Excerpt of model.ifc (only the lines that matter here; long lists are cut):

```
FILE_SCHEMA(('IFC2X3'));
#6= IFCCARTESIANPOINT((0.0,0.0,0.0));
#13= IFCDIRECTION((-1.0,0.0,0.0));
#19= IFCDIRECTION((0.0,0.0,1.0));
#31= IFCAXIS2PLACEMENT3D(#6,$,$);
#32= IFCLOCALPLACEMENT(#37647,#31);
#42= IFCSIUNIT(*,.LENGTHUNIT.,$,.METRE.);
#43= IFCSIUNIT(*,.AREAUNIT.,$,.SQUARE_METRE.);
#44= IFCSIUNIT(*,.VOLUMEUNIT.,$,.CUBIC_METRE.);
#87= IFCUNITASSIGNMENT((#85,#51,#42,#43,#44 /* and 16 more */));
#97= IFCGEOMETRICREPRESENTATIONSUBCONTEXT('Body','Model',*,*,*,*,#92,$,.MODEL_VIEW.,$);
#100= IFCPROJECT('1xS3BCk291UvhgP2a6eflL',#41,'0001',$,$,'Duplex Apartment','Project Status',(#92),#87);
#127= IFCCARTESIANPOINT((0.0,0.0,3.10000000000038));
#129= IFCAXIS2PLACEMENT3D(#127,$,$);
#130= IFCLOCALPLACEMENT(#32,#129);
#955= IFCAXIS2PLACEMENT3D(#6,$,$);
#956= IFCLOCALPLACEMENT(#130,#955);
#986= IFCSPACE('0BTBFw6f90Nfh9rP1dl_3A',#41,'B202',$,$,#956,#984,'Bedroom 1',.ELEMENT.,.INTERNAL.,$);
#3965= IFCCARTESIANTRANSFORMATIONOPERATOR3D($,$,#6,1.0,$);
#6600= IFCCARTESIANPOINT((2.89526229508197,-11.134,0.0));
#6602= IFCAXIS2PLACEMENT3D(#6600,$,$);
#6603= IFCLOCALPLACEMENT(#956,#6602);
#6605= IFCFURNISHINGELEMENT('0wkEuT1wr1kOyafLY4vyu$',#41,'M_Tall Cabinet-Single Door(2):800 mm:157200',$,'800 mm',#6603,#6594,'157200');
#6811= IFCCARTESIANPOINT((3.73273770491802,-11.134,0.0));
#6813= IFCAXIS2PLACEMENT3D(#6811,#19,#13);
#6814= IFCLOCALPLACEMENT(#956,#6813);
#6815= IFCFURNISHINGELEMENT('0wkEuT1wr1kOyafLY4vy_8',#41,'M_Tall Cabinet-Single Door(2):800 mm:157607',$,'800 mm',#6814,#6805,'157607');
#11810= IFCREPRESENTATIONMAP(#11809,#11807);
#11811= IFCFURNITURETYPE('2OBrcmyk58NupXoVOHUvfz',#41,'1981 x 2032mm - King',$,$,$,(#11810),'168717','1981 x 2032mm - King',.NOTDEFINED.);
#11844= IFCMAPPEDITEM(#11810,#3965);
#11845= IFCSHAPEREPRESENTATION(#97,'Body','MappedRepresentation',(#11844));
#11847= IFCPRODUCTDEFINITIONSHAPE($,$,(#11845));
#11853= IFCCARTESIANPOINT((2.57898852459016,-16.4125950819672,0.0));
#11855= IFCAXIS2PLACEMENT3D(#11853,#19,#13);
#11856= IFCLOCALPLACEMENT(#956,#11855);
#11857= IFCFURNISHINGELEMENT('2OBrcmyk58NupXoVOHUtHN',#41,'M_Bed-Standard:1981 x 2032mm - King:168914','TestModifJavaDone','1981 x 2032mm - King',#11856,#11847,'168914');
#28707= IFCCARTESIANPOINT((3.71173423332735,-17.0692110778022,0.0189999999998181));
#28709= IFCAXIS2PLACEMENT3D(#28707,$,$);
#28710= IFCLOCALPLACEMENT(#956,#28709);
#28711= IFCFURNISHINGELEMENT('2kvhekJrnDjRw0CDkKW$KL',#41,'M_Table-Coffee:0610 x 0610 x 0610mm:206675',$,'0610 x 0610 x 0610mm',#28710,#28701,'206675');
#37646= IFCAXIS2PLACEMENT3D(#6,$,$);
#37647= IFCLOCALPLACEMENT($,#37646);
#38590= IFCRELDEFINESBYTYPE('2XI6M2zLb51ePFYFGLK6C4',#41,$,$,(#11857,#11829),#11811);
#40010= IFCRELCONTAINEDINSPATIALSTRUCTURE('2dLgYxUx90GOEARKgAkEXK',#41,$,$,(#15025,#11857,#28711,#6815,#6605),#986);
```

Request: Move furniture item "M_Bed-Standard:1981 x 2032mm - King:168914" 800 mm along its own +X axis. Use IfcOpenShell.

```python
import ifcopenshell
import ifcopenshell.api.geometry
import ifcopenshell.util.placement
import ifcopenshell.util.unit

model = ifcopenshell.open("model.ifc")
unit_scale = ifcopenshell.util.unit.calculate_unit_scale(model)

item = model.by_guid("2OBrcmyk58NupXoVOHUtHN")
matrix = ifcopenshell.util.placement.get_local_placement(item.ObjectPlacement)
matrix[:3, 3] += matrix[:3, 0] * 0.8 / unit_scale
ifcopenshell.api.geometry.edit_object_placement(model, product=item, matrix=matrix, is_si=False)

print(ifcopenshell.util.placement.get_local_placement(item.ObjectPlacement).round(3) + 0.0)

model.write("model_rev.ifc")
```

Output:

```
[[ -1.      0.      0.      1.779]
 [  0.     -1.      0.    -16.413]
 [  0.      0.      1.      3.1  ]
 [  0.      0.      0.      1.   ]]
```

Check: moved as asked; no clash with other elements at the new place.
